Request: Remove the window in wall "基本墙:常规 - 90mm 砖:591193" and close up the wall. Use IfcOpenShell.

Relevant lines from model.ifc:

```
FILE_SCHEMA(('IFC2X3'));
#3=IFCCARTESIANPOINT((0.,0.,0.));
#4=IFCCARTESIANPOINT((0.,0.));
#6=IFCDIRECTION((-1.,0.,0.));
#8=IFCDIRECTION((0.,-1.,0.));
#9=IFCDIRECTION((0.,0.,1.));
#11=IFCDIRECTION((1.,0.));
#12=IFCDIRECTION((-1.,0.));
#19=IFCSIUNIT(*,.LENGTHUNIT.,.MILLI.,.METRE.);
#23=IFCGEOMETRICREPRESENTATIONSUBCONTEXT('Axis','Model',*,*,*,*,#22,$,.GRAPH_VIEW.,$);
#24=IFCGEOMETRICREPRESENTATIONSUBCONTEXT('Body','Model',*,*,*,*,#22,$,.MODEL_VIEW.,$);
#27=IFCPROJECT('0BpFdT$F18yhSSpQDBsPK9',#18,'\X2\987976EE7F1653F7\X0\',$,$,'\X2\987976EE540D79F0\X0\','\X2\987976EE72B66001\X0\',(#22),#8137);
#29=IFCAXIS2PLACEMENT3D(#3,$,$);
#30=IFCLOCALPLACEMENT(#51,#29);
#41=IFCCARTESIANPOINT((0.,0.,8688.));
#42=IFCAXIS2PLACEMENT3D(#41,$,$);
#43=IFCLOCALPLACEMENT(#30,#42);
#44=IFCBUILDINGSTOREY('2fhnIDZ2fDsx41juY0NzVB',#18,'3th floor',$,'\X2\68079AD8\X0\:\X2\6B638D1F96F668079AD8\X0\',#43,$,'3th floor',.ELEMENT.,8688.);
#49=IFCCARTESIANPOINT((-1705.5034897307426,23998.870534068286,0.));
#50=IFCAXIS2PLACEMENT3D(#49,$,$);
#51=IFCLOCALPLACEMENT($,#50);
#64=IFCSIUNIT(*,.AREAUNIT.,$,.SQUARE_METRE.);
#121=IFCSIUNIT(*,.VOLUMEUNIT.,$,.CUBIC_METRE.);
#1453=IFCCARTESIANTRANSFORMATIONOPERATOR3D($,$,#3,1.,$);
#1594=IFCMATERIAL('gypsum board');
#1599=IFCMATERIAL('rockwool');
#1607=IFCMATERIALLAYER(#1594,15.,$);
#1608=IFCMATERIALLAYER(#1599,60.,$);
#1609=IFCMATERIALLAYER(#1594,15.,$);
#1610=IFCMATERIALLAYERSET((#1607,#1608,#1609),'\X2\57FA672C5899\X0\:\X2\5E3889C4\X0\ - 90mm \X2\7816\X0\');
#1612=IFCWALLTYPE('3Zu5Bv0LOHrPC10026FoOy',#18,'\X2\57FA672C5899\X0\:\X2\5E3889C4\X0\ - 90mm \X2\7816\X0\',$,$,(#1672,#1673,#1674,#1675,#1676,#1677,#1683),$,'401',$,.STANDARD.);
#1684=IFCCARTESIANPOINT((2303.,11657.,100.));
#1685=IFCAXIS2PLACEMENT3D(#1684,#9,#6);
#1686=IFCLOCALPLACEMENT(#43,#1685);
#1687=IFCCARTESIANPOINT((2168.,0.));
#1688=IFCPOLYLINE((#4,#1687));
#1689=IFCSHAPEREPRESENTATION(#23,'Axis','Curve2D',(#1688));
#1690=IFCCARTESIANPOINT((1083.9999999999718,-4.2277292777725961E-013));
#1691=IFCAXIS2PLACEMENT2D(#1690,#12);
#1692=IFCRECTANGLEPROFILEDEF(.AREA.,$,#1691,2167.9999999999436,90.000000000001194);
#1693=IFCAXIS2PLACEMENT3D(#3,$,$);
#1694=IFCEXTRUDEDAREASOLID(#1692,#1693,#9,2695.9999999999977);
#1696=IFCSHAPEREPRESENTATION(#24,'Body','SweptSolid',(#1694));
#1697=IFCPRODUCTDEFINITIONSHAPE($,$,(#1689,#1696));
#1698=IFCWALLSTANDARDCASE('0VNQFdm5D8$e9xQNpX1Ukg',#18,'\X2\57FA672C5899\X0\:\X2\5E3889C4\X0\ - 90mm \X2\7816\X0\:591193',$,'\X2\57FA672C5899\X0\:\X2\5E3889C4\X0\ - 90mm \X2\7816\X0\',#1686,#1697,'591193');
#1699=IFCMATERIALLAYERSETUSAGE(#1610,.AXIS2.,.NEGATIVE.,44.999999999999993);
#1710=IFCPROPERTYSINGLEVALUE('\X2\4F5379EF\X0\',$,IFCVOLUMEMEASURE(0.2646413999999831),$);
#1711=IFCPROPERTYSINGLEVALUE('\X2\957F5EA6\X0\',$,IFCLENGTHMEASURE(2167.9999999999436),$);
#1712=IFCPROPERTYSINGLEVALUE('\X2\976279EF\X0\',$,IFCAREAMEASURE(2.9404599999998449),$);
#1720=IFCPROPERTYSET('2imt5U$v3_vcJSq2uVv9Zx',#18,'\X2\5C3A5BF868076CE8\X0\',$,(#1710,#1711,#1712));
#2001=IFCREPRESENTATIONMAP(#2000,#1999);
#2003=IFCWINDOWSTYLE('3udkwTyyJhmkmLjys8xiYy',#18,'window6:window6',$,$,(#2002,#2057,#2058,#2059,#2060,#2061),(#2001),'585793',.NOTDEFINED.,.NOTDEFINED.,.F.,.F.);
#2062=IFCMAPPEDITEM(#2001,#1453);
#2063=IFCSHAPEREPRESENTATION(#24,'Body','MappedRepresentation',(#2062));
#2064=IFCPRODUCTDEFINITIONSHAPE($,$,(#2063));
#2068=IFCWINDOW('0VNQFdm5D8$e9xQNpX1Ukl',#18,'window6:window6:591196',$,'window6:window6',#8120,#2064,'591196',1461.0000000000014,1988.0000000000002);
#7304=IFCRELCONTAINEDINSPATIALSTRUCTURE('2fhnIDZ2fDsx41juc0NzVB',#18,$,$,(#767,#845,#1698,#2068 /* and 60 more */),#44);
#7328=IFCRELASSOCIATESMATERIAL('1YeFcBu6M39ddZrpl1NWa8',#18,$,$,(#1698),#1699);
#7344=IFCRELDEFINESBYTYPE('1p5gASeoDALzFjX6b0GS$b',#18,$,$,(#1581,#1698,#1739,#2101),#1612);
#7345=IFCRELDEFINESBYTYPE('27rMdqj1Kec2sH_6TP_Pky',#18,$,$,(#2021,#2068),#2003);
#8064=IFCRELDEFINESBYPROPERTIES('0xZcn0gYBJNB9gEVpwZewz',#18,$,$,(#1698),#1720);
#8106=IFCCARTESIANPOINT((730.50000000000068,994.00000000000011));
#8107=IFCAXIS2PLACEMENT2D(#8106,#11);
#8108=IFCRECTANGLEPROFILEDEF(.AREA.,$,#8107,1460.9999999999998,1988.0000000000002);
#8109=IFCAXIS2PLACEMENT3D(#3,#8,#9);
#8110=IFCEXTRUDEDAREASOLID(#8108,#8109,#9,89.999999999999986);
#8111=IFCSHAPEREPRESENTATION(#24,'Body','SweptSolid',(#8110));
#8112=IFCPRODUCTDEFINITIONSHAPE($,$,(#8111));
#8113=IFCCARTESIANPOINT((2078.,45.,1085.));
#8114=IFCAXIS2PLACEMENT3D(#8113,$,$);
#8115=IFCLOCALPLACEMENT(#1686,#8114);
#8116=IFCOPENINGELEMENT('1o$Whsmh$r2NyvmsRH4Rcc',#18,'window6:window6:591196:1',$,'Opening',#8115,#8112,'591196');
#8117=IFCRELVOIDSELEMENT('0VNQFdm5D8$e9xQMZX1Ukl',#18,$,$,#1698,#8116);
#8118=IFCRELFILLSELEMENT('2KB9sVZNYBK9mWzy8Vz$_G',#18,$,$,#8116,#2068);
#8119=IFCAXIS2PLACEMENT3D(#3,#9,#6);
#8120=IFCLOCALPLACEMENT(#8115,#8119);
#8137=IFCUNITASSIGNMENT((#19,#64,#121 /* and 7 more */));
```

```python
import ifcopenshell
import ifcopenshell.api.feature
import ifcopenshell.api.pset
import ifcopenshell.api.root
import ifcopenshell.geom
import ifcopenshell.util.element
import ifcopenshell.util.shape
import ifcopenshell.util.unit

model = ifcopenshell.open("model.ifc")
area_scale = ifcopenshell.util.unit.calculate_unit_scale(model, "AREAUNIT")
volume_scale = ifcopenshell.util.unit.calculate_unit_scale(model, "VOLUMEUNIT")
settings = ifcopenshell.geom.settings()


def volume(element):
    """Net volume in cubic metres, openings subtracted."""
    shape = ifcopenshell.geom.create_shape(settings, element)
    return ifcopenshell.util.shape.get_volume(shape.geometry)


window = model.by_id(2068)
opening = window.FillsVoids[0].RelatingOpeningElement
wall = opening.VoidsElements[0].RelatingBuildingElement
before = volume(wall)

ifcopenshell.api.root.remove_product(model, product=window)
ifcopenshell.api.feature.remove_feature(model, feature=opening)

after = volume(wall)
thickness = 0.09  # wall thickness in metres

# Update the wall's stored quantities.
pset = model.by_id(ifcopenshell.util.element.get_pset(wall, "尺寸标注", should_inherit=False)["id"])
ifcopenshell.api.pset.edit_pset(model, pset=pset, properties={
    "体积": model.create_entity("IfcVolumeMeasure", after / volume_scale),
    "面积": model.create_entity("IfcAreaMeasure", after / thickness / area_scale),
})

print(f"wall volume {before:.3f} -> {after:.3f} m3")

model.write("model_rev.ifc")
```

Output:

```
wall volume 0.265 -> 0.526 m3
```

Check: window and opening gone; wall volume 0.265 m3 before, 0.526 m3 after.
